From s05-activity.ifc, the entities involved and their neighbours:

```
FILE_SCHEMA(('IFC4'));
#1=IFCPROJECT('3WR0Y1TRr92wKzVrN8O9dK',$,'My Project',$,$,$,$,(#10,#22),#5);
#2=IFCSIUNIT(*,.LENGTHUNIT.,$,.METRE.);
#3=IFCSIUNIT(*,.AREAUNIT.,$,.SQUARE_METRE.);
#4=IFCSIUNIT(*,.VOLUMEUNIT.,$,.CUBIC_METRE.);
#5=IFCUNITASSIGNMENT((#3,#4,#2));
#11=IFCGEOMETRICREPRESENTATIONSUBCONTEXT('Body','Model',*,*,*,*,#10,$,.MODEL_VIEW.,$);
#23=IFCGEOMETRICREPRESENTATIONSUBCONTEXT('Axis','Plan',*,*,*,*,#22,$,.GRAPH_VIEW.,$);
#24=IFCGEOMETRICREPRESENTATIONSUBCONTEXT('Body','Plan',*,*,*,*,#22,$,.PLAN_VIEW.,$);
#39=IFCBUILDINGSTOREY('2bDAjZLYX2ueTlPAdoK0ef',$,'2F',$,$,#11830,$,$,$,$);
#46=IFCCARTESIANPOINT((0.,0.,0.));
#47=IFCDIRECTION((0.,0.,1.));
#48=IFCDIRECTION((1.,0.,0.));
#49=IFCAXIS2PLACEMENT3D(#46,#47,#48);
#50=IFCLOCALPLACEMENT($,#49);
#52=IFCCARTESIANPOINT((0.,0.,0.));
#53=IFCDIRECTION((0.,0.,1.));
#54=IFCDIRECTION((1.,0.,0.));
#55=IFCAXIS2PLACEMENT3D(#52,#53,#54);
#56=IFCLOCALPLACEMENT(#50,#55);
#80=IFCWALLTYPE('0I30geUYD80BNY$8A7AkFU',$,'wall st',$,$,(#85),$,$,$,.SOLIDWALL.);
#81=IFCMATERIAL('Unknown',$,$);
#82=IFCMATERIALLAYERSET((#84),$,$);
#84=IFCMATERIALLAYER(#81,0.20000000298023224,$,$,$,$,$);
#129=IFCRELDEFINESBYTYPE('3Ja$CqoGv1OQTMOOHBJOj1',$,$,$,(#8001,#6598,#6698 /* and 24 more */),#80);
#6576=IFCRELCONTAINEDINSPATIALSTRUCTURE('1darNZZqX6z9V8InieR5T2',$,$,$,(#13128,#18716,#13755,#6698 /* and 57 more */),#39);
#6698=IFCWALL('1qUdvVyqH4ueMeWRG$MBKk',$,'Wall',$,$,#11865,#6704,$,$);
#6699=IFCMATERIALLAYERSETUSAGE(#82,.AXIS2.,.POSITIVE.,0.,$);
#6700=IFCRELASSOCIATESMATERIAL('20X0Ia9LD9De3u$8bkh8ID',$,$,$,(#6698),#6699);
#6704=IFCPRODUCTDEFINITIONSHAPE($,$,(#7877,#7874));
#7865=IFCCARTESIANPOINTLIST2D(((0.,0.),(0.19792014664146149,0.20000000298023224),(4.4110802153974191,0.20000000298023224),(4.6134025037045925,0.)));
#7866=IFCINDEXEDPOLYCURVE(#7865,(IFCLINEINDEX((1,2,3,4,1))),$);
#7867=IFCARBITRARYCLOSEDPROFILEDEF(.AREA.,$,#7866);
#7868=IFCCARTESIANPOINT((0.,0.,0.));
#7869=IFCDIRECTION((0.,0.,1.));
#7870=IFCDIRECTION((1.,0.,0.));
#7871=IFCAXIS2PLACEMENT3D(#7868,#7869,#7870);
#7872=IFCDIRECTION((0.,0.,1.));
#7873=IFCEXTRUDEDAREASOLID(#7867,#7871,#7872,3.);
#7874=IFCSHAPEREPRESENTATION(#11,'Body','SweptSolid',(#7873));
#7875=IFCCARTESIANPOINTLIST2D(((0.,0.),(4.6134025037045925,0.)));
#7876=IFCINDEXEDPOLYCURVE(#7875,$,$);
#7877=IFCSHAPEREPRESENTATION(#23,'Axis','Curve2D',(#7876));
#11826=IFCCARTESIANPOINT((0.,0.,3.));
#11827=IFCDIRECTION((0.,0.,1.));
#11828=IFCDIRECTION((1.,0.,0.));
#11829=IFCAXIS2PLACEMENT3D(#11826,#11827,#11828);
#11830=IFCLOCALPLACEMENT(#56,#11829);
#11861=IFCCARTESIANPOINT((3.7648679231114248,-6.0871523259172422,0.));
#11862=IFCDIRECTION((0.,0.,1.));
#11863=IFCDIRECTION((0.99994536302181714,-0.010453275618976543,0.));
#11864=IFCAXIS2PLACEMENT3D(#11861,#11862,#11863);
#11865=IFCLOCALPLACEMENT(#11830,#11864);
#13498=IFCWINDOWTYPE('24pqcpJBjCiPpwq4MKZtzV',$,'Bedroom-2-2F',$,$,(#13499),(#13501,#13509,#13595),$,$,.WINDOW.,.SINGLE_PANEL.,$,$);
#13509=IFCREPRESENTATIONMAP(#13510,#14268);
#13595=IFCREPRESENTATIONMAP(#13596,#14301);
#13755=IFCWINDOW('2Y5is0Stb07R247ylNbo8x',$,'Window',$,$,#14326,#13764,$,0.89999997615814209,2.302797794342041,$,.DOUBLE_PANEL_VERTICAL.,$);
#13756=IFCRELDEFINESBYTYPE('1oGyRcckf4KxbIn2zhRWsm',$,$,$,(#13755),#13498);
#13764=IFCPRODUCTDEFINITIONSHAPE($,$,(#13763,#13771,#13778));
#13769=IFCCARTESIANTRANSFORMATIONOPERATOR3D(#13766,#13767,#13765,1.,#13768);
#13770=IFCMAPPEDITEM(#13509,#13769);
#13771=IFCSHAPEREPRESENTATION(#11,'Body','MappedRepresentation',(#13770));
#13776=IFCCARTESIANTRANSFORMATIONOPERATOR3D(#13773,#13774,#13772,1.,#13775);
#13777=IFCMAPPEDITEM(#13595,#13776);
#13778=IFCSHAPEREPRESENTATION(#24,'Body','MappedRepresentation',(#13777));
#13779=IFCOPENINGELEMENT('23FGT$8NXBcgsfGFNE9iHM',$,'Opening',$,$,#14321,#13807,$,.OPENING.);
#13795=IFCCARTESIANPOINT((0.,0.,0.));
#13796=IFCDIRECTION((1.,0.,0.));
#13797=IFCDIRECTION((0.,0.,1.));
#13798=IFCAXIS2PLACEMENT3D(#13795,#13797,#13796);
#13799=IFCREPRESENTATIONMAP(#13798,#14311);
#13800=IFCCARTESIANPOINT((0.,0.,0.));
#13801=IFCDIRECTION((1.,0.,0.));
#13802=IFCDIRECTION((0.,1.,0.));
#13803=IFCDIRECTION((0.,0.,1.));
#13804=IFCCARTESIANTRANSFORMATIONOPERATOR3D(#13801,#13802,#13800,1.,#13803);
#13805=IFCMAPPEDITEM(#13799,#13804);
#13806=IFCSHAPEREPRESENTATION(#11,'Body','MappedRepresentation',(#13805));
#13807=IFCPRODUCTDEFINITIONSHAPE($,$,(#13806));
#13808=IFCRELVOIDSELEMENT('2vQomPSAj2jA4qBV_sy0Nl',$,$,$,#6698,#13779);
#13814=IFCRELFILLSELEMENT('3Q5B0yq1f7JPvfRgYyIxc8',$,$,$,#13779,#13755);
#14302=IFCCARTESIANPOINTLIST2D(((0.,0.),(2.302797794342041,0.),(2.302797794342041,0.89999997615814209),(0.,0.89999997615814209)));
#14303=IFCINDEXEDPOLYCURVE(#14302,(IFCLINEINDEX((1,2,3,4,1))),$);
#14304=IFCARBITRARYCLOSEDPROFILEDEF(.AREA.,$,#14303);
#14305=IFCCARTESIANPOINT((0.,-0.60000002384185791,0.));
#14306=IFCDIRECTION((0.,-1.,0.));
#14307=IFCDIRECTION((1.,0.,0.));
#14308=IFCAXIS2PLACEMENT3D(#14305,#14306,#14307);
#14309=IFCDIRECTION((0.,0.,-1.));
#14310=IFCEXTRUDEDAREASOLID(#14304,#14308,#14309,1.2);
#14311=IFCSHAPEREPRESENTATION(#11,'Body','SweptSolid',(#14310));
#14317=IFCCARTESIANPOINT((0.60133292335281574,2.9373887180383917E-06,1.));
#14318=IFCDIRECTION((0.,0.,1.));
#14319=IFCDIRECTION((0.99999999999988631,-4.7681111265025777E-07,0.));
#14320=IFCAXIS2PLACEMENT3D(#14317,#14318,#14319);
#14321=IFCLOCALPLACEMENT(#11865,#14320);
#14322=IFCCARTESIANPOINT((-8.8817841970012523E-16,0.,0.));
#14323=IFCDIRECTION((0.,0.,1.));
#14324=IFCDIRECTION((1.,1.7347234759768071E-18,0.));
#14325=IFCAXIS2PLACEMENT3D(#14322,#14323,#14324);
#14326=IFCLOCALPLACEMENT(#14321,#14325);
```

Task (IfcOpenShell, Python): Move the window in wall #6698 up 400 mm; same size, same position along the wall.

```python
import numpy as np
import ifcopenshell
import ifcopenshell.api.geometry
import ifcopenshell.util.placement
import ifcopenshell.util.unit

model = ifcopenshell.open("s05-activity.ifc")
unit_scale = ifcopenshell.util.unit.calculate_unit_scale(model)

window = model.by_id(13755)
opening = window.FillsVoids[0].RelatingOpeningElement
dz = 0.4 / unit_scale

shift = np.array([0.0, 0.0, dz])
# The window is placed relative to its opening, so it follows when the opening moves.
matrix = ifcopenshell.util.placement.get_local_placement(opening.ObjectPlacement)
matrix[:3, 3] += shift
ifcopenshell.api.geometry.edit_object_placement(
    model, product=opening, matrix=matrix, is_si=False, should_transform_children=True
)

print(f"moved by {dz * unit_scale:+.3f} m")

model.write("s05-activity_rev.ifc")
```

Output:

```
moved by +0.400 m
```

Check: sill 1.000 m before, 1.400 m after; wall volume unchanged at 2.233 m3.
